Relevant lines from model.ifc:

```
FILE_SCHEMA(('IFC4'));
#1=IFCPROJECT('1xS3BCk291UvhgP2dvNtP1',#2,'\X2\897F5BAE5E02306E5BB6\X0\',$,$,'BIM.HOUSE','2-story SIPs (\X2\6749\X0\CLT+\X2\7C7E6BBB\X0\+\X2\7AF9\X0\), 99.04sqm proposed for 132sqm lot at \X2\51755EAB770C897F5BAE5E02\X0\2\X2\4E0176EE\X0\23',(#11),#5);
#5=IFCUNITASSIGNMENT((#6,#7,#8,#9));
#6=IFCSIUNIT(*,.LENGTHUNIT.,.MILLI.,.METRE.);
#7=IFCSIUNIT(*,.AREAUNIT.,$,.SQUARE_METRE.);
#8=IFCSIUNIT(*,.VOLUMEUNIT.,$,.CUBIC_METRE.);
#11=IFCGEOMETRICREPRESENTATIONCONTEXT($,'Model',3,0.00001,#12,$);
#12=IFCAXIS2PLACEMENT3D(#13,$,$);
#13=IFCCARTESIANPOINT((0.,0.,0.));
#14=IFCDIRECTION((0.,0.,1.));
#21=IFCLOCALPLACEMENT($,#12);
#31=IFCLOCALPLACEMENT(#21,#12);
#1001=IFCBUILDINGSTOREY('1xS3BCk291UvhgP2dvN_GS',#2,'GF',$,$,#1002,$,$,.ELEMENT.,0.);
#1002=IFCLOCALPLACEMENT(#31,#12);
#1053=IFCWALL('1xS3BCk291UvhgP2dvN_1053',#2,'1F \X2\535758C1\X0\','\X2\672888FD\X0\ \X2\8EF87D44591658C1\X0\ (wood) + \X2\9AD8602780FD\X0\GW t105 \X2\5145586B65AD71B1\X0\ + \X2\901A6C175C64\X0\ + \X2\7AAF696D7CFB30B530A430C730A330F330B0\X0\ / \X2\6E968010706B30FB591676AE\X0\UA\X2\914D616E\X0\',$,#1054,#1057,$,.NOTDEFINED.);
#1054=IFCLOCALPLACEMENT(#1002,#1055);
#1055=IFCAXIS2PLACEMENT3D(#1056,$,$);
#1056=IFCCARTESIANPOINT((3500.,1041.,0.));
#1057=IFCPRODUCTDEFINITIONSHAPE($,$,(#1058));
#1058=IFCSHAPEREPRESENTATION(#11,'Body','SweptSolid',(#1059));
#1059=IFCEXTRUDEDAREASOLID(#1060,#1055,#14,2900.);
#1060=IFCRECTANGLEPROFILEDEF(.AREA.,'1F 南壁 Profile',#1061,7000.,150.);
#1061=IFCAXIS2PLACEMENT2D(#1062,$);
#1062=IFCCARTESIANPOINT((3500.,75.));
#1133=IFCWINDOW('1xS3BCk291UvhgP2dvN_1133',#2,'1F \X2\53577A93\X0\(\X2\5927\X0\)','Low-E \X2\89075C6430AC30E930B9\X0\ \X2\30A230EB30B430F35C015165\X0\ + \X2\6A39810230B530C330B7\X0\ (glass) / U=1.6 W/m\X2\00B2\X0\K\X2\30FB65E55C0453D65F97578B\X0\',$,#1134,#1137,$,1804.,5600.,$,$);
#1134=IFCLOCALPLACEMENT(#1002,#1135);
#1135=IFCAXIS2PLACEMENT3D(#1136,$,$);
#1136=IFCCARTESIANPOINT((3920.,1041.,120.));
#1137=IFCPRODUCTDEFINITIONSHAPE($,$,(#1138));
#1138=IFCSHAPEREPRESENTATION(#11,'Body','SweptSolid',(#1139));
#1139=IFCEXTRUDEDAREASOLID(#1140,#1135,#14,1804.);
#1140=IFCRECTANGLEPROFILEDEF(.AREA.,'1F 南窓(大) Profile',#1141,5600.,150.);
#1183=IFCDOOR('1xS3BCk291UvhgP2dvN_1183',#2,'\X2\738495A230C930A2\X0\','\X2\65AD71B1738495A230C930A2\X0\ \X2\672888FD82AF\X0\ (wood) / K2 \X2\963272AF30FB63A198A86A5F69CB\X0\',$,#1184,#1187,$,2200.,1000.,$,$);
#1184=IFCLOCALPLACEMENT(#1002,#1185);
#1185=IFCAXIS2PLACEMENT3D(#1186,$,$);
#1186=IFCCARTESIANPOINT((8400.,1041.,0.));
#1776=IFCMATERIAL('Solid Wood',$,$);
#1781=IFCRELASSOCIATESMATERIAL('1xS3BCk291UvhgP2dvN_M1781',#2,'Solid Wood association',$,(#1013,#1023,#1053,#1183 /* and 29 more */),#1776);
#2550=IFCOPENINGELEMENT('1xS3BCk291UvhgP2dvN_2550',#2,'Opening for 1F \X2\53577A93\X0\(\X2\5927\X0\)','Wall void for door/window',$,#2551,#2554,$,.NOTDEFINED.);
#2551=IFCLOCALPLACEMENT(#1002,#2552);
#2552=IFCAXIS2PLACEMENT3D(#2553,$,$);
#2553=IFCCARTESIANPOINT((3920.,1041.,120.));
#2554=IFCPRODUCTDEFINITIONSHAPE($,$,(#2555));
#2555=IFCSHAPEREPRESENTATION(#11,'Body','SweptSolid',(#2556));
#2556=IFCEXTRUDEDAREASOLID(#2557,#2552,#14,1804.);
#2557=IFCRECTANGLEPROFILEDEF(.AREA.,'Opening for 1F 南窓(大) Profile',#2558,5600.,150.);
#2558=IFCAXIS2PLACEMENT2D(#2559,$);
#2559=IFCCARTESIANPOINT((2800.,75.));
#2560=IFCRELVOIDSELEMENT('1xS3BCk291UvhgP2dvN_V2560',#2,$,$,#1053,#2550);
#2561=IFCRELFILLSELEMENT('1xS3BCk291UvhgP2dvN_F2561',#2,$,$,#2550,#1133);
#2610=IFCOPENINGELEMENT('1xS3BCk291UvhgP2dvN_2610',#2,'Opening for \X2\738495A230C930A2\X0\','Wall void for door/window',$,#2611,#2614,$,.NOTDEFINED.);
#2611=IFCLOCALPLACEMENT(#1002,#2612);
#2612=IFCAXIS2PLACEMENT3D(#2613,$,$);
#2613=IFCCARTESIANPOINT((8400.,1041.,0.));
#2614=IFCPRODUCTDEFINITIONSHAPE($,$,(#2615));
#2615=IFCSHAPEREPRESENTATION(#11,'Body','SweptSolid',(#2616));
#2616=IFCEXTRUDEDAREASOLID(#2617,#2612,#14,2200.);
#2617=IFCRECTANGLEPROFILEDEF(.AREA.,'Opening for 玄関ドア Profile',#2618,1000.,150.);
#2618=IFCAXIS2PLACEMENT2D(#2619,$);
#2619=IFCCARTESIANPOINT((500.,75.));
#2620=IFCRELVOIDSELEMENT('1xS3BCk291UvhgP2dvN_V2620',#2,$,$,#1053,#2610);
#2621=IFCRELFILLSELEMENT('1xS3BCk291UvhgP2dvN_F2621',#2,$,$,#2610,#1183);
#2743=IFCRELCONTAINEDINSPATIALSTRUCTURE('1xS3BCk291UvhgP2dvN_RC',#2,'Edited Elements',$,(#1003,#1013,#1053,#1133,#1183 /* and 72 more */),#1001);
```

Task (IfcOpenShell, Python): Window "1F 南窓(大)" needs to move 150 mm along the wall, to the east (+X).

```python
import ifcopenshell
import ifcopenshell.api.geometry
import ifcopenshell.util.placement
import ifcopenshell.util.unit

model = ifcopenshell.open("model.ifc")
unit_scale = ifcopenshell.util.unit.calculate_unit_scale(model)

window = model.by_guid("1xS3BCk291UvhgP2dvN_1133")
opening = window.FillsVoids[0].RelatingOpeningElement
wall = opening.VoidsElements[0].RelatingBuildingElement

wall_matrix = ifcopenshell.util.placement.get_local_placement(wall.ObjectPlacement)
shift = wall_matrix[:3, 0] * 0.15 / unit_scale
before = ifcopenshell.util.placement.get_local_placement(window.ObjectPlacement)[:3, 3].copy()

# The window is not placed relative to its opening, so move both.
for product in (opening, window):
    matrix = ifcopenshell.util.placement.get_local_placement(product.ObjectPlacement)
    matrix[:3, 3] += shift
    ifcopenshell.api.geometry.edit_object_placement(model, product=product, matrix=matrix, is_si=False)

after = ifcopenshell.util.placement.get_local_placement(window.ObjectPlacement)[:3, 3]
print("window moved by", (after - before).round(3) + 0.0)

model.write("model-out.ifc")
```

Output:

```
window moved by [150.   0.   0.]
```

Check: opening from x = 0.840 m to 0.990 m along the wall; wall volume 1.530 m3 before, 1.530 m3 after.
